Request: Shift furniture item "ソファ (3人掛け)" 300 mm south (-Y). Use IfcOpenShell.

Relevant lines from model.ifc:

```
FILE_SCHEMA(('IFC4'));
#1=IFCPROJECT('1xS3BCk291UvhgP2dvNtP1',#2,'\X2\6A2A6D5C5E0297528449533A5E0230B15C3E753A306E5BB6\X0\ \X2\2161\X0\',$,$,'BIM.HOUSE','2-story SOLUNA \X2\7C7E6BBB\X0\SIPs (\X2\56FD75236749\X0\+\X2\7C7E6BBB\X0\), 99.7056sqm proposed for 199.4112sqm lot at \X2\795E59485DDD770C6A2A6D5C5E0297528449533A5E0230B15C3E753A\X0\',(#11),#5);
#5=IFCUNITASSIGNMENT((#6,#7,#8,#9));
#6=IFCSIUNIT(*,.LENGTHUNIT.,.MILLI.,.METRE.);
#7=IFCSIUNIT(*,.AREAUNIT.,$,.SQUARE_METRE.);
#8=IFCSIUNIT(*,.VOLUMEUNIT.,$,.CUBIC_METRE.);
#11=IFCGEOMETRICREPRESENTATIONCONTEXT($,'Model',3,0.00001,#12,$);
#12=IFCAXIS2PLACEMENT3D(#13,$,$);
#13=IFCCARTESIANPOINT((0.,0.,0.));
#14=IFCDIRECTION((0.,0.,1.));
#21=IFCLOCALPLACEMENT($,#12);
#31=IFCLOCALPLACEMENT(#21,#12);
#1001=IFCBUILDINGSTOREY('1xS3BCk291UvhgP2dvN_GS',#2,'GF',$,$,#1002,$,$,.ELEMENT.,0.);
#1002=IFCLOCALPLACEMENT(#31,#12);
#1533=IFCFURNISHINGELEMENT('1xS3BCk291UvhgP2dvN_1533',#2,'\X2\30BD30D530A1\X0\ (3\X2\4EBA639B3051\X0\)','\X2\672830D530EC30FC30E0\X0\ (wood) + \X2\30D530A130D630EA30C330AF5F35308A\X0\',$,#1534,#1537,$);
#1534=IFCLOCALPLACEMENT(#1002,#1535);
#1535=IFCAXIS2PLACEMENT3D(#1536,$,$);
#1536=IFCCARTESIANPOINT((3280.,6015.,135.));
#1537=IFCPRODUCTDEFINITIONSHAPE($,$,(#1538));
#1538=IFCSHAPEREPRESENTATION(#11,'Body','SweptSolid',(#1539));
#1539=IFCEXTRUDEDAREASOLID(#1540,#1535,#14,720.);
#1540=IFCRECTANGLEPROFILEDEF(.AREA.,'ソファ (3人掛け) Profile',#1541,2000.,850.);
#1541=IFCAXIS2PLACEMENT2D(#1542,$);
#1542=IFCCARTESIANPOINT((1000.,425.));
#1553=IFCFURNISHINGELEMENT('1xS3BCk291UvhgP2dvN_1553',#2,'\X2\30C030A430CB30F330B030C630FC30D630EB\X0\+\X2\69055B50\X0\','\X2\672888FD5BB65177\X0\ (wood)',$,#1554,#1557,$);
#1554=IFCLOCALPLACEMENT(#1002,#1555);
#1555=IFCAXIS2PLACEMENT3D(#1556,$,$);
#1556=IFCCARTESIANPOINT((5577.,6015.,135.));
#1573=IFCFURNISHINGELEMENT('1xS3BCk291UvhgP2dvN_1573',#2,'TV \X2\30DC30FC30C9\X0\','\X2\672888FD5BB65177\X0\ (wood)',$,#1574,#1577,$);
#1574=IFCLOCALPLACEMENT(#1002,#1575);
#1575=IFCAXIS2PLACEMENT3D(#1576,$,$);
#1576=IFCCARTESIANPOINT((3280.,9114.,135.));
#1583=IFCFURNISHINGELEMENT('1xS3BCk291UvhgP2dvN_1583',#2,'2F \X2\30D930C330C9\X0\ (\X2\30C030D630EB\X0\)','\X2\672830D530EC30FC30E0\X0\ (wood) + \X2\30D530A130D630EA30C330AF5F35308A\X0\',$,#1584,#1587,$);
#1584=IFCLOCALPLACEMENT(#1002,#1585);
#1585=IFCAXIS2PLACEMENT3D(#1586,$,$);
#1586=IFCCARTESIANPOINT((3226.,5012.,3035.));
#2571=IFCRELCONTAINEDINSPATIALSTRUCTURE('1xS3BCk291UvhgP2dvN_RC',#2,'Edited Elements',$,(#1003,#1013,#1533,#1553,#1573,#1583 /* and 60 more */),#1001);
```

```python
import ifcopenshell
import ifcopenshell.api.geometry
import ifcopenshell.util.placement
import ifcopenshell.util.unit

model = ifcopenshell.open("model.ifc")
unit_scale = ifcopenshell.util.unit.calculate_unit_scale(model)

item = model.by_guid("1xS3BCk291UvhgP2dvN_1533")
matrix = ifcopenshell.util.placement.get_local_placement(item.ObjectPlacement)
matrix[1, 3] -= 0.3 / unit_scale
ifcopenshell.api.geometry.edit_object_placement(model, product=item, matrix=matrix, is_si=False)

print(ifcopenshell.util.placement.get_local_placement(item.ObjectPlacement).round(3) + 0.0)

model.write("model_updated.ifc")
```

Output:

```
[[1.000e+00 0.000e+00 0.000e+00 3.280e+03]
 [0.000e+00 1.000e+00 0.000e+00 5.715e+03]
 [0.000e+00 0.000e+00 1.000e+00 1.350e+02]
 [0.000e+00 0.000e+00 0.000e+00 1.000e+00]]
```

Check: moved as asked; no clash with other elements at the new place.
